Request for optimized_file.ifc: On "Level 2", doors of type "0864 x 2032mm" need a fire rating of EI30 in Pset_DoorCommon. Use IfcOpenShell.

First a look at what the model holds.

```python
import ifcopenshell
import ifcopenshell.util.element

model = ifcopenshell.open("optimized_file.ifc")
print(model.schema)
storey = next(s for s in model.by_type("IfcBuildingStorey") if s.Name == "Level 2")
doors = [e for e in ifcopenshell.util.element.get_decomposition(storey) if e.is_a("IfcDoor")]
seen = {}
for e in doors:
    element_type = ifcopenshell.util.element.get_type(e)
    key = (element_type.Name if element_type != e and element_type else None, ifcopenshell.util.element.get_pset(e, "Pset_DoorCommon", "FireRating"))
    seen[key] = seen.get(key, 0) + 1
for (name, value), count in sorted(seen.items(), key=str):
    print(count, "x", name, "|", value)
```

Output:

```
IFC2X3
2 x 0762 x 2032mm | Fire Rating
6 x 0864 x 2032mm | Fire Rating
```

```python
import ifcopenshell
import ifcopenshell.api.pset
import ifcopenshell.util.element

model = ifcopenshell.open("optimized_file.ifc")

storey = next(s for s in model.by_type("IfcBuildingStorey") if s.Name == "Level 2")
doors = [e for e in ifcopenshell.util.element.get_decomposition(storey) if e.is_a("IfcDoor")]

count = 0
for e in doors:
    element_type = ifcopenshell.util.element.get_type(e)
    if element_type in (None, e) or element_type.Name != "0864 x 2032mm":
        continue
    # add_pset returns the element's existing set when there is one.
    pset = ifcopenshell.api.pset.add_pset(model, product=e, name="Pset_DoorCommon")
    ifcopenshell.api.pset.edit_pset(model, pset=pset, properties={"FireRating": "EI30"})
    count += 1

print(count, "doors updated")

model.write("optimized_file_v2.ifc")
```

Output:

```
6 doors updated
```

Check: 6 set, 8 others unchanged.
